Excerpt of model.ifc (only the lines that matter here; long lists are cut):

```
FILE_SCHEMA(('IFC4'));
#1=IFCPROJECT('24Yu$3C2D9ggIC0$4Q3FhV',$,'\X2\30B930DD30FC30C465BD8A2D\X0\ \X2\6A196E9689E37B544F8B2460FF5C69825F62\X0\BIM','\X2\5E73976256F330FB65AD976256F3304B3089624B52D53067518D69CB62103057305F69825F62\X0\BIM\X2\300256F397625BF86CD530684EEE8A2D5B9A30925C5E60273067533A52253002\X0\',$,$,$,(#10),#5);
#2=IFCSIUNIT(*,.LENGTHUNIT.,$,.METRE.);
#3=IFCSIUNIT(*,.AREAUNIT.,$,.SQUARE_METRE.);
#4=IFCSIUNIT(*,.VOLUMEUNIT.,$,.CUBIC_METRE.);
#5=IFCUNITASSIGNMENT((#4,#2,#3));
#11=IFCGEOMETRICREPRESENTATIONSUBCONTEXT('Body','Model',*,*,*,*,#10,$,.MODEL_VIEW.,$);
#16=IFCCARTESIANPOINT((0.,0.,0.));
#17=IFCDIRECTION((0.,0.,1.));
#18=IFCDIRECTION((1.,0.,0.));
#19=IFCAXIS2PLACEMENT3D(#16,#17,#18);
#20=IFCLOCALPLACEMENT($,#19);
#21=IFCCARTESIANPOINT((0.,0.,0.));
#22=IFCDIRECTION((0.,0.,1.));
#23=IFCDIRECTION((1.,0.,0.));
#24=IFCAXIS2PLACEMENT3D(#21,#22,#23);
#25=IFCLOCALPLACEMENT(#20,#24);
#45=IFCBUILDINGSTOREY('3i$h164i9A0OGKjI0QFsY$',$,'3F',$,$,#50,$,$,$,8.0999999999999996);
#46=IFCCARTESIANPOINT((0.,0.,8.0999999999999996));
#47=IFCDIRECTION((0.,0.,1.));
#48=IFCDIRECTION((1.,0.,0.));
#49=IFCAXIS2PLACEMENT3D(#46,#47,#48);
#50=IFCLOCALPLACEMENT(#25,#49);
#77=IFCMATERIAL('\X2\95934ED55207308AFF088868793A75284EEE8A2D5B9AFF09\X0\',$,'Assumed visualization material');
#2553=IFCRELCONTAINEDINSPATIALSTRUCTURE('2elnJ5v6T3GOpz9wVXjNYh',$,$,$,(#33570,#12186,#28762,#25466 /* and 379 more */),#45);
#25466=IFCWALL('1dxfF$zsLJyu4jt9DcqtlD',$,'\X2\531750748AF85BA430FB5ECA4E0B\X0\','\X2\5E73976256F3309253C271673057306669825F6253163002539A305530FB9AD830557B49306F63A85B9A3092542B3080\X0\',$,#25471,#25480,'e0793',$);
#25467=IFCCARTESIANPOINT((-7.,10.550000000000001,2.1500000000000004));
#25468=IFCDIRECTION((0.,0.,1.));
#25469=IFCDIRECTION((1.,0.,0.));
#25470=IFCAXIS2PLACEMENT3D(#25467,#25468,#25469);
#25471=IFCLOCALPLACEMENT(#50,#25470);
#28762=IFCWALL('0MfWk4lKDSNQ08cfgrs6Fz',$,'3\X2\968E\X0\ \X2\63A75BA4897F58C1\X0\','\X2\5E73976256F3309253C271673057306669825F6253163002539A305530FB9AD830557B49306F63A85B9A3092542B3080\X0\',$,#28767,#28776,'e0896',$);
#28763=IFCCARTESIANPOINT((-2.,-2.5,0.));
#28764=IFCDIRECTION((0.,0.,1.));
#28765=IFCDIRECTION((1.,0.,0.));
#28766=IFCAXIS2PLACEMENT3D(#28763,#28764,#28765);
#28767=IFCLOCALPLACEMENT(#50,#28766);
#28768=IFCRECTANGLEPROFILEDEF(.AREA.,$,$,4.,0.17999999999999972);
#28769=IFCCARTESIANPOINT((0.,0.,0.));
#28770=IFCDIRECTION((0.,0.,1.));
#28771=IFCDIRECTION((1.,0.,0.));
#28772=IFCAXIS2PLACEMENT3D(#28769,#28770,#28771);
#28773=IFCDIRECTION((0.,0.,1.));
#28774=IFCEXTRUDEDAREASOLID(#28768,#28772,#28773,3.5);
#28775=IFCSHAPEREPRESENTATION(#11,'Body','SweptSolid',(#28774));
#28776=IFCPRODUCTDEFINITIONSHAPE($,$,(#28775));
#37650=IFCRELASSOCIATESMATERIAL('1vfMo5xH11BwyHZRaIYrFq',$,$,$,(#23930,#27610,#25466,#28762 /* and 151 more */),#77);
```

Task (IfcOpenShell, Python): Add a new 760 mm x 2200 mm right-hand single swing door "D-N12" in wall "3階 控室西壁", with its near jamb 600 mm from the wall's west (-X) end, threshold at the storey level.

```python
import numpy as np
import ifcopenshell
import ifcopenshell.api.feature
import ifcopenshell.api.geometry
import ifcopenshell.api.root
import ifcopenshell.api.spatial
import ifcopenshell.geom
import ifcopenshell.util.element
import ifcopenshell.util.placement
import ifcopenshell.util.representation
import ifcopenshell.util.shape
import ifcopenshell.util.unit

model = ifcopenshell.open("model.ifc")
unit_scale = ifcopenshell.util.unit.calculate_unit_scale(model)
settings = ifcopenshell.geom.settings()


def volume(element):
    """Net volume in cubic metres, openings subtracted."""
    shape = ifcopenshell.geom.create_shape(settings, element)
    return ifcopenshell.util.shape.get_volume(shape.geometry)


wall = model.by_id(28762)
storey = ifcopenshell.util.element.get_container(wall, ifc_class="IfcBuildingStorey")
context = ifcopenshell.util.representation.get_context(model, "Model", "Body", "MODEL_VIEW")
before = volume(wall)

width, height, from_end, sill = 0.76, 2.2, 0.6, 0.0  # metres

# The wall runs along its own X axis, and the end named is its -X end.
wall_shape = ifcopenshell.geom.create_shape(settings, wall)
x, y, z = ifcopenshell.util.shape.get_vertices(wall_shape.geometry).T
start = x.min() + from_end
face, thickness = float(y.min()), float(y.max() - y.min())
wall_matrix = ifcopenshell.util.placement.get_local_placement(wall.ObjectPlacement)
level = ifcopenshell.util.placement.get_local_placement(storey.ObjectPlacement)[2, 3]


def in_wall(x, y):
    """Placement at x, y metres in the wall's axes, at sill height."""
    matrix = wall_matrix.copy()
    matrix[:, 3] = wall_matrix @ np.array([x / unit_scale, y / unit_scale, 0.0, 1.0])
    matrix[2, 3] = level + sill / unit_scale
    return matrix


# Opening: a box that overshoots both wall faces by 50 mm.
opening = ifcopenshell.api.root.create_entity(model, ifc_class="IfcOpeningElement", predefined_type="OPENING")
box = ifcopenshell.api.geometry.add_wall_representation(
    model, context=context, length=width, height=height, thickness=thickness + 0.1
)
ifcopenshell.api.geometry.assign_representation(model, product=opening, representation=box)
ifcopenshell.api.geometry.edit_object_placement(model, product=opening, matrix=in_wall(start, face - 0.05), is_si=False)
ifcopenshell.api.feature.add_feature(model, feature=opening, element=wall)

door = ifcopenshell.api.root.create_entity(model, ifc_class="IfcDoor", name="D-N12", predefined_type="DOOR")
door.OverallWidth, door.OverallHeight = width / unit_scale, height / unit_scale
door.OperationType = "SINGLE_SWING_RIGHT"
body = ifcopenshell.api.geometry.add_door_representation(
    model,
    context=context,
    overall_width=door.OverallWidth,
    overall_height=door.OverallHeight,
    operation_type="SINGLE_SWING_RIGHT",
    lining_properties={"LiningDepth": thickness / unit_scale, "ThresholdDepth": thickness / unit_scale},
)
ifcopenshell.api.geometry.assign_representation(model, product=door, representation=body)
ifcopenshell.api.spatial.assign_container(model, products=[door], relating_structure=storey)
ifcopenshell.api.feature.add_filling(model, opening=opening, element=door)

# The lining spans the wall, so the door starts at the wall face.
ifcopenshell.api.geometry.edit_object_placement(model, product=door, matrix=in_wall(start, face), is_si=False)

after = volume(wall)

print(f"wall volume {before:.3f} -> {after:.3f} m3")

model.write("model_edited.ifc")
```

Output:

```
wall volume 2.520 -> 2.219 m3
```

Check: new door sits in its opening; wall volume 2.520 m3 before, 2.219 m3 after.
